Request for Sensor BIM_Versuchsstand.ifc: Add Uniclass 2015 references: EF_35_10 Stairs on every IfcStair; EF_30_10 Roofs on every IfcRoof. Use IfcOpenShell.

First a look at what the model holds.

```python
import ifcopenshell

model = ifcopenshell.open("Sensor BIM_Versuchsstand.ifc")
print(model.schema)
print("classifications:", [c.Name for c in model.by_type("IfcClassification")])
for ifc_class in ("IfcDoor", "IfcRoof", "IfcStair", "IfcWall", "IfcWindow"):
    print(ifc_class, len(model.by_type(ifc_class)))
```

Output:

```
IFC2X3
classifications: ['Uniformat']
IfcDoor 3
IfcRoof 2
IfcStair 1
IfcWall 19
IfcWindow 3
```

```python
import ifcopenshell
import ifcopenshell.api.classification

model = ifcopenshell.open("Sensor BIM_Versuchsstand.ifc")

# IFC2X3 requires Source and Edition and has no link from the project to the system.
system = model.create_entity("IfcClassification", Source="NBS", Edition="2015", Name="Uniclass 2015")

codes = {
    "IfcStair": ("EF_35_10", "Stairs"),
    "IfcRoof": ("EF_30_10", "Roofs"),
}
for ifc_class, (code, name) in codes.items():
    products = model.by_type(ifc_class)
    ifcopenshell.api.classification.add_reference(
        model, products=products, classification=system, identification=code, name=name
    )
    print(code, len(products))

model.write("Sensor BIM_Versuchsstand-out.ifc")
```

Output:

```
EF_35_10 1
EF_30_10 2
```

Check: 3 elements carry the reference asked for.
